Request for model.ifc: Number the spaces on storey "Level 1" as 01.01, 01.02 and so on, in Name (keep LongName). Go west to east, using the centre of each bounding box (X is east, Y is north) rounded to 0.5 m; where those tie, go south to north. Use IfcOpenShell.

First a look at what the model holds.

```python
import ifcopenshell
import ifcopenshell.util.element
import ifcopenshell.util.placement

model = ifcopenshell.open("model.ifc")
print(model.schema)
storey = next(s for s in model.by_type("IfcBuildingStorey") if s.Name == "Level 1")
spaces = [e for e in ifcopenshell.util.element.get_decomposition(storey) if e.is_a("IfcSpace")]
for e in sorted(spaces, key=lambda e: e.id()):
    origin = ifcopenshell.util.placement.get_local_placement(e.ObjectPlacement)[:3, 3]
    print(e.id(), e.Name, e.LongName, origin.round(2) + 0.0, sep=" | ")
```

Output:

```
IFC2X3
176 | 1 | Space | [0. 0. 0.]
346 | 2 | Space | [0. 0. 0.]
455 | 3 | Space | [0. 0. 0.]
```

```python
import ifcopenshell
import ifcopenshell.geom
import ifcopenshell.util.element
import ifcopenshell.util.shape

model = ifcopenshell.open("model.ifc")
settings = ifcopenshell.geom.settings()
settings.set("use-world-coords", True)


def centre(element):
    shape = ifcopenshell.geom.create_shape(settings, element)
    return ifcopenshell.util.shape.get_bbox_centroid(shape.geometry)


storey = next(s for s in model.by_type("IfcBuildingStorey") if s.Name == "Level 1")
spaces = [e for e in ifcopenshell.util.element.get_decomposition(storey) if e.is_a("IfcSpace")]

# Insertion points can sit at a corner or the storey origin, so sort by the geometry (in metres).
centres = {e: centre(e) for e in spaces}
spaces.sort(key=lambda e: (round(centres[e][0] / 0.5), centres[e][1]))

for i, e in enumerate(spaces, start=1):
    number = f"01.{i:02d}"
    e.Name = number
    print(e.id(), number)

model.write("model-out.ifc")
```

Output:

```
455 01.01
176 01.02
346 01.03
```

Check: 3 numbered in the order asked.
